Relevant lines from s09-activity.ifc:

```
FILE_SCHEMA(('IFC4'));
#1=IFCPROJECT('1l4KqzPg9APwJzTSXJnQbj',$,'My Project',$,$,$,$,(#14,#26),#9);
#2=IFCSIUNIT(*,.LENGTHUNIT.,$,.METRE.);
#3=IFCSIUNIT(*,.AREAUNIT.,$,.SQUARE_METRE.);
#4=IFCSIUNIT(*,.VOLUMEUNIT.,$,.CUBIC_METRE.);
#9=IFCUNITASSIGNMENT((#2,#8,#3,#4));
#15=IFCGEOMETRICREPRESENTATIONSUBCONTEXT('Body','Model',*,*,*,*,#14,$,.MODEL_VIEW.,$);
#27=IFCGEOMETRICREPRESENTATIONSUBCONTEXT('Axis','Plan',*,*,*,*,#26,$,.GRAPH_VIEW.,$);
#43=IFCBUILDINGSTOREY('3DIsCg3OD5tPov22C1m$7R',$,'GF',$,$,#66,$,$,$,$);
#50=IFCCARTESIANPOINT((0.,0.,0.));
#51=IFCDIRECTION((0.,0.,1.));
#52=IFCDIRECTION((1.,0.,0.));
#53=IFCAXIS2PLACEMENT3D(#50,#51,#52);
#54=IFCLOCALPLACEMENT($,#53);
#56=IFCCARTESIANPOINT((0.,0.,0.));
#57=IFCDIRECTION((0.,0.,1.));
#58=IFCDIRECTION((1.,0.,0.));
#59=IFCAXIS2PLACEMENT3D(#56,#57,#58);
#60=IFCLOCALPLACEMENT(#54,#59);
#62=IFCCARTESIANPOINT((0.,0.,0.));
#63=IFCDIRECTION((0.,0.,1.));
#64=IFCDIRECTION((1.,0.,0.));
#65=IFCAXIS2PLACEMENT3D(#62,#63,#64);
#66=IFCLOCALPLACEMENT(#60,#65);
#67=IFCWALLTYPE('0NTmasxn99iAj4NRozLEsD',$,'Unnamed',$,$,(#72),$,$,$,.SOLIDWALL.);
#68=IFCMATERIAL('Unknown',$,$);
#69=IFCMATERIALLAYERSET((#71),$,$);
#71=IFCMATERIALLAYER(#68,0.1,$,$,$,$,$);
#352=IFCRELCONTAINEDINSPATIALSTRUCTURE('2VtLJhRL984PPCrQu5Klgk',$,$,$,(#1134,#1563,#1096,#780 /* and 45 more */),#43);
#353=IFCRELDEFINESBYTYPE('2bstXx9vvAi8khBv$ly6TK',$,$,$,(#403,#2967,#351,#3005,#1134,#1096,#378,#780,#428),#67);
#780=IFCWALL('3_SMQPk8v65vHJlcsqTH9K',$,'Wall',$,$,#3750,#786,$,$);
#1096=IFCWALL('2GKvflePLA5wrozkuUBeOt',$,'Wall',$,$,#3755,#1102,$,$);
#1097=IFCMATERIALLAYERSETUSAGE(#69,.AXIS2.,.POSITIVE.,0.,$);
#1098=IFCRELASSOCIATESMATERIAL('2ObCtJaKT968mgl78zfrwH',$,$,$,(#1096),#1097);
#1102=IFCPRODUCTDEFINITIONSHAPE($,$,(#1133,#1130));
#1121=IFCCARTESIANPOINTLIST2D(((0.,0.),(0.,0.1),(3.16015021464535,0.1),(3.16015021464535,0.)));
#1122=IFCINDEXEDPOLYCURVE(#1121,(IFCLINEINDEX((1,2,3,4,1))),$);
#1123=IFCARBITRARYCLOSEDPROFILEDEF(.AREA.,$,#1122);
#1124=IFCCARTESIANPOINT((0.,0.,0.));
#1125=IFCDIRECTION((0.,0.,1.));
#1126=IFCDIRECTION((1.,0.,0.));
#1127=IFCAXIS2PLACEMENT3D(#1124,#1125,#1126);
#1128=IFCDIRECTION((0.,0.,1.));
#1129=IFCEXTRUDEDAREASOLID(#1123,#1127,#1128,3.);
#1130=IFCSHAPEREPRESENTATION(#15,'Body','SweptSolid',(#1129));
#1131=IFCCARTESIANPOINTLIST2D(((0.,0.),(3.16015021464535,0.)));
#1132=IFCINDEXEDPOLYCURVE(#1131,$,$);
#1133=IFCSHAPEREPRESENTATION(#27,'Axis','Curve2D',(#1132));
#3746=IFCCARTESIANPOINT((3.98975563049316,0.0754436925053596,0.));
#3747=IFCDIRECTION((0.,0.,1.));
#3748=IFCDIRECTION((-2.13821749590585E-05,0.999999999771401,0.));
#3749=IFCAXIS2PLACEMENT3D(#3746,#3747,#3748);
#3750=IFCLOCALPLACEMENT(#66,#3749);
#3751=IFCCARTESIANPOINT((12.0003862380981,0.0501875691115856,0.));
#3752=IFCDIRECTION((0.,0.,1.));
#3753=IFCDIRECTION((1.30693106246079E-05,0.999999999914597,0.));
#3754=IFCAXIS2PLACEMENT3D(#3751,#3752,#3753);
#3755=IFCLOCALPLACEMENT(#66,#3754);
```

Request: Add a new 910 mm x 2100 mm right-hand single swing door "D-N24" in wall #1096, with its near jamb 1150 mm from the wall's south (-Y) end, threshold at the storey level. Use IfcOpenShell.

```python
import numpy as np
import ifcopenshell
import ifcopenshell.api.feature
import ifcopenshell.api.geometry
import ifcopenshell.api.root
import ifcopenshell.api.spatial
import ifcopenshell.geom
import ifcopenshell.util.element
import ifcopenshell.util.placement
import ifcopenshell.util.representation
import ifcopenshell.util.shape
import ifcopenshell.util.unit

model = ifcopenshell.open("s09-activity.ifc")
unit_scale = ifcopenshell.util.unit.calculate_unit_scale(model)
settings = ifcopenshell.geom.settings()


def volume(element):
    """Net volume in cubic metres, openings subtracted."""
    shape = ifcopenshell.geom.create_shape(settings, element)
    return ifcopenshell.util.shape.get_volume(shape.geometry)


wall = model.by_guid("2GKvflePLA5wrozkuUBeOt")
storey = ifcopenshell.util.element.get_container(wall, ifc_class="IfcBuildingStorey")
context = ifcopenshell.util.representation.get_context(model, "Model", "Body", "MODEL_VIEW")
before = volume(wall)

width, height, from_end, sill = 0.91, 2.1, 1.15, 0.0  # metres

# The wall runs along its own X axis, and the end named is its -X end.
wall_shape = ifcopenshell.geom.create_shape(settings, wall)
x, y, z = ifcopenshell.util.shape.get_vertices(wall_shape.geometry).T
start = x.min() + from_end
face, thickness = float(y.min()), float(y.max() - y.min())
wall_matrix = ifcopenshell.util.placement.get_local_placement(wall.ObjectPlacement)
level = ifcopenshell.util.placement.get_local_placement(storey.ObjectPlacement)[2, 3]


def in_wall(x, y):
    """Placement at x, y metres in the wall's axes, at sill height."""
    matrix = wall_matrix.copy()
    matrix[:, 3] = wall_matrix @ np.array([x / unit_scale, y / unit_scale, 0.0, 1.0])
    matrix[2, 3] = level + sill / unit_scale
    return matrix


# Opening: a box that overshoots both wall faces by 50 mm.
opening = ifcopenshell.api.root.create_entity(model, ifc_class="IfcOpeningElement", predefined_type="OPENING")
box = ifcopenshell.api.geometry.add_wall_representation(
    model, context=context, length=width, height=height, thickness=thickness + 0.1
)
ifcopenshell.api.geometry.assign_representation(model, product=opening, representation=box)
ifcopenshell.api.geometry.edit_object_placement(model, product=opening, matrix=in_wall(start, face - 0.05), is_si=False)
ifcopenshell.api.feature.add_feature(model, feature=opening, element=wall)

door = ifcopenshell.api.root.create_entity(model, ifc_class="IfcDoor", name="D-N24", predefined_type="DOOR")
door.OverallWidth, door.OverallHeight = width / unit_scale, height / unit_scale
door.OperationType = "SINGLE_SWING_RIGHT"
body = ifcopenshell.api.geometry.add_door_representation(
    model,
    context=context,
    overall_width=door.OverallWidth,
    overall_height=door.OverallHeight,
    operation_type="SINGLE_SWING_RIGHT",
    lining_properties={"LiningDepth": thickness / unit_scale, "ThresholdDepth": thickness / unit_scale},
)
ifcopenshell.api.geometry.assign_representation(model, product=door, representation=body)
ifcopenshell.api.spatial.assign_container(model, products=[door], relating_structure=storey)
ifcopenshell.api.feature.add_filling(model, opening=opening, element=door)

# The lining spans the wall, so the door starts at the wall face.
ifcopenshell.api.geometry.edit_object_placement(model, product=door, matrix=in_wall(start, face), is_si=False)

after = volume(wall)

print(f"wall volume {before:.3f} -> {after:.3f} m3")

model.write("s09-activity_v2.ifc")
```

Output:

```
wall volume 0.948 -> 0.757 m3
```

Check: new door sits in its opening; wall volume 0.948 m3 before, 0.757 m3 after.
